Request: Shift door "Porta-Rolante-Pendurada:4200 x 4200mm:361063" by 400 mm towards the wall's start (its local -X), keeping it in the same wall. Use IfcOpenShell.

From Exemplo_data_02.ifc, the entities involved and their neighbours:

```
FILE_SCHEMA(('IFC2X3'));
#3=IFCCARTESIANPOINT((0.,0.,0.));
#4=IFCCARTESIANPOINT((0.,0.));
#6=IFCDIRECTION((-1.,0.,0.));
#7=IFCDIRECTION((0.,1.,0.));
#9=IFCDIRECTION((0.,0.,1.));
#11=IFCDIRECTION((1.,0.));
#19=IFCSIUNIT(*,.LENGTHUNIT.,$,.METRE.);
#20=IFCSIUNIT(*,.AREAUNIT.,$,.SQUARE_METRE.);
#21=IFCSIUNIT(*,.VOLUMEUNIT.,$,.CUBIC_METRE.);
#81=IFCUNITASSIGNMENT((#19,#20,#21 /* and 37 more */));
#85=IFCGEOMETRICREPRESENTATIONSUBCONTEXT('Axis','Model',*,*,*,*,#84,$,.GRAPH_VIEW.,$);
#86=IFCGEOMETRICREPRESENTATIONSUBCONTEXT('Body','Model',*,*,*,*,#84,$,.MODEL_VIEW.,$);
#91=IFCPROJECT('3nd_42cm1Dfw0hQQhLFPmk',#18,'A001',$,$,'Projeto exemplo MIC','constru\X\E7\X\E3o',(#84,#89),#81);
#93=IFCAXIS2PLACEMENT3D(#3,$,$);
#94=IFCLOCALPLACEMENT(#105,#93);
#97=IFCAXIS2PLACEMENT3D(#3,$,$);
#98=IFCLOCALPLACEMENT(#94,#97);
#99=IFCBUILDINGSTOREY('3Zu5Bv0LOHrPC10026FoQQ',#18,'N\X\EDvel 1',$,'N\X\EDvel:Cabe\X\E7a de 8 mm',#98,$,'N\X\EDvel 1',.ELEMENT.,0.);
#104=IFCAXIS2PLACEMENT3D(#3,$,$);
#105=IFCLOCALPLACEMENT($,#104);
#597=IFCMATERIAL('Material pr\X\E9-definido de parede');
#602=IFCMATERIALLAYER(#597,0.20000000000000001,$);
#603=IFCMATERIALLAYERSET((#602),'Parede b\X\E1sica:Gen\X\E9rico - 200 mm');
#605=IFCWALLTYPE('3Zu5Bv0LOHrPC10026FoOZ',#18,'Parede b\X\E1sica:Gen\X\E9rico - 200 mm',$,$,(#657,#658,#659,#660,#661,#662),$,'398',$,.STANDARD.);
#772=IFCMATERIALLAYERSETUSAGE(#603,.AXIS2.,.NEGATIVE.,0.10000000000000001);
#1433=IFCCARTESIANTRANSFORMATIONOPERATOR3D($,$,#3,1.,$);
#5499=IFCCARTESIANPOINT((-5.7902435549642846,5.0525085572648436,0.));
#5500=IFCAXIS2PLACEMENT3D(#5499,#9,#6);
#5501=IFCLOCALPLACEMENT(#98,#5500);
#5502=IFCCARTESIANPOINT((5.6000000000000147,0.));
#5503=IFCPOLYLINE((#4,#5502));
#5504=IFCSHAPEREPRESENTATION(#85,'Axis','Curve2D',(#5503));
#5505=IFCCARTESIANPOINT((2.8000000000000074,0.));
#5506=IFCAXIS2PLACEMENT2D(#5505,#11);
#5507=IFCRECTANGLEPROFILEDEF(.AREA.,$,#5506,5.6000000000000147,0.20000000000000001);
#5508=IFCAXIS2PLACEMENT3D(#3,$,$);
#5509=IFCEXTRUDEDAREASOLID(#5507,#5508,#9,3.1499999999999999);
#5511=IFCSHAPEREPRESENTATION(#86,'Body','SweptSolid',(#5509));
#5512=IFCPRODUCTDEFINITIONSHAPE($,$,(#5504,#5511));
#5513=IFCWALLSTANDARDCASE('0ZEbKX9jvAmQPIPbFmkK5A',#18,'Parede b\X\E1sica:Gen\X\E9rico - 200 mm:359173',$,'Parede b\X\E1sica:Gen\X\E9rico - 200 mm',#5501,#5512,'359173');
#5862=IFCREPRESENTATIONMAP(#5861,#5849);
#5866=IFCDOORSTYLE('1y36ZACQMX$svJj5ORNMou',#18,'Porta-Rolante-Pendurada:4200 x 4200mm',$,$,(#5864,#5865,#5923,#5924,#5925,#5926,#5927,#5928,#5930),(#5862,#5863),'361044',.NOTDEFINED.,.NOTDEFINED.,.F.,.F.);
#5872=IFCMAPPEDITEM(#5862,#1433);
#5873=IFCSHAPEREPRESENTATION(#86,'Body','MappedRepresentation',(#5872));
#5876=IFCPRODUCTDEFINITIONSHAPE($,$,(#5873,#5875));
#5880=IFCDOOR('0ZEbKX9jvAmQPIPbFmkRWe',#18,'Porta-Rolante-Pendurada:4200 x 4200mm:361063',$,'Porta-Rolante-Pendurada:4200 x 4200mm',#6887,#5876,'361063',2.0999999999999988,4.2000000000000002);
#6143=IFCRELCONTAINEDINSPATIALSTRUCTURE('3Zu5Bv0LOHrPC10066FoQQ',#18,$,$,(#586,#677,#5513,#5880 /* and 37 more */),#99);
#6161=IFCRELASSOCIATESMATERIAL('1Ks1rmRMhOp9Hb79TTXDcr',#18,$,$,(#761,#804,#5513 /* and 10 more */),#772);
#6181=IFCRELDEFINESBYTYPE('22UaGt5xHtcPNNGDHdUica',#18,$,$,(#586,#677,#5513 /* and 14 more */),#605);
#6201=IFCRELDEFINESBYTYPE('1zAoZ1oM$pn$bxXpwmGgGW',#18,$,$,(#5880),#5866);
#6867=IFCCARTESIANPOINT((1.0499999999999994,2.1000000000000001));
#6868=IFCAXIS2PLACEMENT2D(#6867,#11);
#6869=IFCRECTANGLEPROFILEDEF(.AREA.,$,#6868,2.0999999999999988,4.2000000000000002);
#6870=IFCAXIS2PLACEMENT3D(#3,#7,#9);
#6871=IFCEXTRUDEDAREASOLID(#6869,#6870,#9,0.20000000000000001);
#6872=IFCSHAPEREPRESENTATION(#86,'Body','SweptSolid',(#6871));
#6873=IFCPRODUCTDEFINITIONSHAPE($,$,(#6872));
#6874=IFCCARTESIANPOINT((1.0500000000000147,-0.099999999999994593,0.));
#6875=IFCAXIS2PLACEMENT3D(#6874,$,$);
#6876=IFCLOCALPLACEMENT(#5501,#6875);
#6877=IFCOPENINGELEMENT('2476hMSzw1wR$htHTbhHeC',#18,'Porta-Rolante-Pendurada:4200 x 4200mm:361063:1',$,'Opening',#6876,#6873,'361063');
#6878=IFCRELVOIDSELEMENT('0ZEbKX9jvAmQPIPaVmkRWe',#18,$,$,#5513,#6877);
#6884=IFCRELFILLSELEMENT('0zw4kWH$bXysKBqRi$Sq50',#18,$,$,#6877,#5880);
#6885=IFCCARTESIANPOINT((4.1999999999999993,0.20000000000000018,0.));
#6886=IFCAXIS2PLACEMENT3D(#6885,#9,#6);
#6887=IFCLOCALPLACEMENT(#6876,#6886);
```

```python
import ifcopenshell
import ifcopenshell.api.geometry
import ifcopenshell.util.placement
import ifcopenshell.util.unit

model = ifcopenshell.open("Exemplo_data_02.ifc")
unit_scale = ifcopenshell.util.unit.calculate_unit_scale(model)

door = model.by_guid("0ZEbKX9jvAmQPIPbFmkRWe")
opening = door.FillsVoids[0].RelatingOpeningElement
wall = opening.VoidsElements[0].RelatingBuildingElement

wall_matrix = ifcopenshell.util.placement.get_local_placement(wall.ObjectPlacement)
shift = wall_matrix[:3, 0] * -0.4 / unit_scale
before = ifcopenshell.util.placement.get_local_placement(door.ObjectPlacement)[:3, 3].copy()

# The door is placed relative to its opening, so it follows when the opening moves.
matrix = ifcopenshell.util.placement.get_local_placement(opening.ObjectPlacement)
matrix[:3, 3] += shift
ifcopenshell.api.geometry.edit_object_placement(
    model, product=opening, matrix=matrix, is_si=False, should_transform_children=True
)

after = ifcopenshell.util.placement.get_local_placement(door.ObjectPlacement)[:3, 3]
print("door moved by", (after - before).round(3) + 0.0)

model.write("Exemplo_data_02-out.ifc")
```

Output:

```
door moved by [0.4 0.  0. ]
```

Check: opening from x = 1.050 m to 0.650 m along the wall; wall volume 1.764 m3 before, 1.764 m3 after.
